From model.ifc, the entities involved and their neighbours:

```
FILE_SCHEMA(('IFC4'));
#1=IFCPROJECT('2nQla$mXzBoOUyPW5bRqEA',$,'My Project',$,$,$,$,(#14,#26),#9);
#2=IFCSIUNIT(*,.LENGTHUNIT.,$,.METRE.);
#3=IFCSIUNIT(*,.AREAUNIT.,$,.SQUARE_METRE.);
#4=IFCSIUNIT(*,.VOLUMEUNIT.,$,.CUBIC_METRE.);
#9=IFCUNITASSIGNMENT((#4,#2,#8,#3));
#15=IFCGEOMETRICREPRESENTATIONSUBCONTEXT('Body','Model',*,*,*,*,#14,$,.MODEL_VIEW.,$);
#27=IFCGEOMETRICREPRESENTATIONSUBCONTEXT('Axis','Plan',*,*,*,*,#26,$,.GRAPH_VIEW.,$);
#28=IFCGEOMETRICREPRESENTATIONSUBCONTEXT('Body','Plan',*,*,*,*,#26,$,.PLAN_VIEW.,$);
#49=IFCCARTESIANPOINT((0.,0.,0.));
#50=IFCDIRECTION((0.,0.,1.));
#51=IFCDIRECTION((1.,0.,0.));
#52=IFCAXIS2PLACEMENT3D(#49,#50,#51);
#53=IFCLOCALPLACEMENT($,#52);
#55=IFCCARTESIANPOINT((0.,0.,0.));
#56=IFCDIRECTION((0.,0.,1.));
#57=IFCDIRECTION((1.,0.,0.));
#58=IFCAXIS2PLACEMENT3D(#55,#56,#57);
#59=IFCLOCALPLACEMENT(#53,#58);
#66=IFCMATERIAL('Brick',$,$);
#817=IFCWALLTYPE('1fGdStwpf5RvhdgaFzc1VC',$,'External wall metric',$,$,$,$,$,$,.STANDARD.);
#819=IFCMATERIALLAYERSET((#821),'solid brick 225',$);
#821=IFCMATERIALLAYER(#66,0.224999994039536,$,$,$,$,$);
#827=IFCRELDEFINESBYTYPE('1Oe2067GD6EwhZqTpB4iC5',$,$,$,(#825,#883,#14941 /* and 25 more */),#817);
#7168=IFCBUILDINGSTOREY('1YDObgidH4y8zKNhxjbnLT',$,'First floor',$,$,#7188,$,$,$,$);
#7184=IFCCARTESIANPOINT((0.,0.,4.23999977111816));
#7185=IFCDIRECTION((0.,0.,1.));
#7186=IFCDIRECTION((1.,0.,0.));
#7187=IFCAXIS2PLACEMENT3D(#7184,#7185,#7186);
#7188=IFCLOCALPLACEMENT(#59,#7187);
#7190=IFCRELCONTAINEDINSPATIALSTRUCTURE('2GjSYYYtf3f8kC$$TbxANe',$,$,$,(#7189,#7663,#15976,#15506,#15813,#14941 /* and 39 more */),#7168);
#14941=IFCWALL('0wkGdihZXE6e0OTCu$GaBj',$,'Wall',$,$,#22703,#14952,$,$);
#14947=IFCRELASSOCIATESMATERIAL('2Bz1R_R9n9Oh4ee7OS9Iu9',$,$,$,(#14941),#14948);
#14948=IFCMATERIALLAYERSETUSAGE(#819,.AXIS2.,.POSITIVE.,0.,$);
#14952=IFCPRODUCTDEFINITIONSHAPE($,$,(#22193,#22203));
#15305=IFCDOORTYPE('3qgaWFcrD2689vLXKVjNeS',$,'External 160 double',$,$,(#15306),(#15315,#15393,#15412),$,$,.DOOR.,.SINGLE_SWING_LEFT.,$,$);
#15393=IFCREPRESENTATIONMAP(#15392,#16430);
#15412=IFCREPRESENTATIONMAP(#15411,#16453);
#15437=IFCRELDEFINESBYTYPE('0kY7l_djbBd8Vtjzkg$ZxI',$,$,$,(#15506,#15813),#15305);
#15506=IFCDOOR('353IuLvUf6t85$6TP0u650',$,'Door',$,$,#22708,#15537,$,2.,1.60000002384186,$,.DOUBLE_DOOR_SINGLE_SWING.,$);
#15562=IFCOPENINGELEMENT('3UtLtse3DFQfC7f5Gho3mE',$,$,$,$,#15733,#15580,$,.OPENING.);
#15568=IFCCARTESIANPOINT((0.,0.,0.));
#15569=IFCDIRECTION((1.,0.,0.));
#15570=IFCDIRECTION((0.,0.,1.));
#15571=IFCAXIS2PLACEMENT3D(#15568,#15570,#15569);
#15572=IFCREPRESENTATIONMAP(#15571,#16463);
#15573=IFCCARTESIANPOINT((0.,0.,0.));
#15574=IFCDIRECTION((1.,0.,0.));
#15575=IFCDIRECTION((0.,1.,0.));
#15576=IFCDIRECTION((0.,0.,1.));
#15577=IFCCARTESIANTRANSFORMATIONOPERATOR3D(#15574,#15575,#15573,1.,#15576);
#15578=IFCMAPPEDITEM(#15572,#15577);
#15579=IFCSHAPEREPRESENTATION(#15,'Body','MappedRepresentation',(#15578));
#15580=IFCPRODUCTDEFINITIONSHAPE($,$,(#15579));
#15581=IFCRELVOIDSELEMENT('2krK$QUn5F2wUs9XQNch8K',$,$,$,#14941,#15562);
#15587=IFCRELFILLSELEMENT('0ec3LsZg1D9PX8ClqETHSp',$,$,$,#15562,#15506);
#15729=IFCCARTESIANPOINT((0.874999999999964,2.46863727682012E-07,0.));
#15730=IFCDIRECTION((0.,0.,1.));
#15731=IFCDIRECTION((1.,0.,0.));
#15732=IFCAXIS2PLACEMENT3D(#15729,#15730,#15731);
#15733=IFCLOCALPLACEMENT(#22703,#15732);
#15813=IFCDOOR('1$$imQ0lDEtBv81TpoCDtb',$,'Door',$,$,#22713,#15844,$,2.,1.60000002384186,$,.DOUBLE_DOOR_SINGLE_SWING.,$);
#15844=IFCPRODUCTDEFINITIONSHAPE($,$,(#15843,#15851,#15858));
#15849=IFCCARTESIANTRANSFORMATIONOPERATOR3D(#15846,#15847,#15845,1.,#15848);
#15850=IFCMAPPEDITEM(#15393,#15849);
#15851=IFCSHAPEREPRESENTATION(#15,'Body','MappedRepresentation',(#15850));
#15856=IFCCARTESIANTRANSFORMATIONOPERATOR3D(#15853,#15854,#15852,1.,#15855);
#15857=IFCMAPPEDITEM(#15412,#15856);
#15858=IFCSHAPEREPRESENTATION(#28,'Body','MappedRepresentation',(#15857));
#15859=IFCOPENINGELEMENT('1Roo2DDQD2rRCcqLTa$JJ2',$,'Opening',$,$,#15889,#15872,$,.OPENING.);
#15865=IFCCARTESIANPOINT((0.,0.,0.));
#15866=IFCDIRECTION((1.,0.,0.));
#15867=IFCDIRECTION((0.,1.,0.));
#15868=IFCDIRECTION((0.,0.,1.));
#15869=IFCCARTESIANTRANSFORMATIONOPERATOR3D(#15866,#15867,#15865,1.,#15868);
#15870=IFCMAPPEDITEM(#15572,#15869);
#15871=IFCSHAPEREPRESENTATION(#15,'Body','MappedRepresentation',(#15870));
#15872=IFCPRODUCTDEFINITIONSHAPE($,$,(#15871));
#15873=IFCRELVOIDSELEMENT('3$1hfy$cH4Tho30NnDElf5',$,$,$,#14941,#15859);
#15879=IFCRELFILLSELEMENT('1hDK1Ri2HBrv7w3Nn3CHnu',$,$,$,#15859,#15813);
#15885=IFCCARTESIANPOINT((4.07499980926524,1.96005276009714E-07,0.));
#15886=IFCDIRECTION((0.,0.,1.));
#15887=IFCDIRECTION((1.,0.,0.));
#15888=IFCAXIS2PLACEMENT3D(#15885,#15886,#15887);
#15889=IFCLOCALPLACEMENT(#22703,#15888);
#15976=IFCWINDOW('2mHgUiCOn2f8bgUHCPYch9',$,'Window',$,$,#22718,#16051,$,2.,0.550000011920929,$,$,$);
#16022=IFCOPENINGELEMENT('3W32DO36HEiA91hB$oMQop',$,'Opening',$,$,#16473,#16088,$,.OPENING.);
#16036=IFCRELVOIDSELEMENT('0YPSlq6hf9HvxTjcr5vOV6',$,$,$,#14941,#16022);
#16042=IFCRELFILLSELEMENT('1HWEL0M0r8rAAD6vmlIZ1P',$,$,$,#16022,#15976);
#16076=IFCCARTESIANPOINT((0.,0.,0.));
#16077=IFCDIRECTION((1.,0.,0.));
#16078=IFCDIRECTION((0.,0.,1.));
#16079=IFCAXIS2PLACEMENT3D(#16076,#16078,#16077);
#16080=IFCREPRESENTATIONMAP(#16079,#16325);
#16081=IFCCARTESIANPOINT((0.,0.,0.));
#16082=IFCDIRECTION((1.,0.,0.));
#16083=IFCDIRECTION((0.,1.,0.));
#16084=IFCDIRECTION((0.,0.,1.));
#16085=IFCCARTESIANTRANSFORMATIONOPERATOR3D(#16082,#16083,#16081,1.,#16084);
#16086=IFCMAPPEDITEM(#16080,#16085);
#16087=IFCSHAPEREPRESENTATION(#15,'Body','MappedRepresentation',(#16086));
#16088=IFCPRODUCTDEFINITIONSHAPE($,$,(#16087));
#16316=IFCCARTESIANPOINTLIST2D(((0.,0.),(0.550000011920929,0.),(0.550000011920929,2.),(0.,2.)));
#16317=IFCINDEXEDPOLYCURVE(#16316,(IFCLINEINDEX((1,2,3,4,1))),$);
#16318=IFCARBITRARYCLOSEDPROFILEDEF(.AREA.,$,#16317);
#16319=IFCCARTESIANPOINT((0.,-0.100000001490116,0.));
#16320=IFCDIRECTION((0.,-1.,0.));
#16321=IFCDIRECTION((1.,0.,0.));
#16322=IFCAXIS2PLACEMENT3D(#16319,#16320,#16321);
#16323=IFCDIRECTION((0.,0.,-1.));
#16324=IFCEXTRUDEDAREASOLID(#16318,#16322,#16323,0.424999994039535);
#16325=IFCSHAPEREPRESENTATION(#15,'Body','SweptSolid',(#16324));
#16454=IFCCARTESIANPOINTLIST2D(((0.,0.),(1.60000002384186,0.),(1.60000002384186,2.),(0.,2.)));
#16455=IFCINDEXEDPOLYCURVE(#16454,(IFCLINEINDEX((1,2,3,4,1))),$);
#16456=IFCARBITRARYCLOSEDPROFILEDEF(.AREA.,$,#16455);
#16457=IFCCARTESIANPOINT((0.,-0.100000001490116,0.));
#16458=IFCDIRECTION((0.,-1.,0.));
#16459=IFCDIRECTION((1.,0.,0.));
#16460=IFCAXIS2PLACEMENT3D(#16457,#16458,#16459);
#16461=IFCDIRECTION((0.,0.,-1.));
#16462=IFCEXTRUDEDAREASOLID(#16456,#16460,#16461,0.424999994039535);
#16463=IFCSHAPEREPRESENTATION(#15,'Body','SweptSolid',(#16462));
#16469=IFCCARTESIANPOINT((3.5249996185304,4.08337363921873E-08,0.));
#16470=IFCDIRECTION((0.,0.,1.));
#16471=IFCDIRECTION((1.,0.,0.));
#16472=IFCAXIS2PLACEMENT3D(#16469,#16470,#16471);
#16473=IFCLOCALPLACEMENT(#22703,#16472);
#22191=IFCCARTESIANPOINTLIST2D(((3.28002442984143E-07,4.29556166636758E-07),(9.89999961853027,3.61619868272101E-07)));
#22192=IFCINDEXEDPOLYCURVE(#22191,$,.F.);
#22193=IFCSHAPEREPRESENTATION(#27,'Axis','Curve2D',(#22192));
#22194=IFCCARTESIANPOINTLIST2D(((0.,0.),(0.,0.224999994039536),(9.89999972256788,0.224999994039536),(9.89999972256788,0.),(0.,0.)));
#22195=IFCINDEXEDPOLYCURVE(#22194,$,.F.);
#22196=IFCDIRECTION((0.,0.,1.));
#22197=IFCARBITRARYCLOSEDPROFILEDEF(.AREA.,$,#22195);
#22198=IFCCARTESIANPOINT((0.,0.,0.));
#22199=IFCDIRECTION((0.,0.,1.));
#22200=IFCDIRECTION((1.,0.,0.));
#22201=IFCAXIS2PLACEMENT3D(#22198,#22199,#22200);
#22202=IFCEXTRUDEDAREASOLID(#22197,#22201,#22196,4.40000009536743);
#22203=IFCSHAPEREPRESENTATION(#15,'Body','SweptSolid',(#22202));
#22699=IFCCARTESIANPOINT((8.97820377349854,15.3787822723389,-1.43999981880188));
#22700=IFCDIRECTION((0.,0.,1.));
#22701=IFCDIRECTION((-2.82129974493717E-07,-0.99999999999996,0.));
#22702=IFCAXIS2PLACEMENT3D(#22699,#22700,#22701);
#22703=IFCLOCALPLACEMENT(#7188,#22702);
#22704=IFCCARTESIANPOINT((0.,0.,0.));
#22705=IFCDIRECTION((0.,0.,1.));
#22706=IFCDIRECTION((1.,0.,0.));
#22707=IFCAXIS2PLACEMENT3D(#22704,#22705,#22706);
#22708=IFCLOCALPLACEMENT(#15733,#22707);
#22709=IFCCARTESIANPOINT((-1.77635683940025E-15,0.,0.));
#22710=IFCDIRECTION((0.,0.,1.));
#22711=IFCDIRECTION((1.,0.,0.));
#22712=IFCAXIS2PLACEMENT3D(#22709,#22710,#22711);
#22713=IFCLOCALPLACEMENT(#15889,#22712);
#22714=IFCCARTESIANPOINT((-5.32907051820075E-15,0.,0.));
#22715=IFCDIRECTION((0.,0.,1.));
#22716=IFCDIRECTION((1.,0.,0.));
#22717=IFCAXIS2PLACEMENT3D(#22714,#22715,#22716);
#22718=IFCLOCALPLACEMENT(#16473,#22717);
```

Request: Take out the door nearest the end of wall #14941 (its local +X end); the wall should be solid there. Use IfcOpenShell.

```python
import ifcopenshell
import ifcopenshell.api.feature
import ifcopenshell.api.root
import ifcopenshell.geom
import ifcopenshell.util.shape

model = ifcopenshell.open("model.ifc")
settings = ifcopenshell.geom.settings()


def volume(element):
    """Net volume in cubic metres, openings subtracted."""
    shape = ifcopenshell.geom.create_shape(settings, element)
    return ifcopenshell.util.shape.get_volume(shape.geometry)


door = model.by_guid("1$$imQ0lDEtBv81TpoCDtb")
opening = door.FillsVoids[0].RelatingOpeningElement
wall = opening.VoidsElements[0].RelatingBuildingElement
before = volume(wall)

ifcopenshell.api.root.remove_product(model, product=door)
ifcopenshell.api.feature.remove_feature(model, feature=opening)

after = volume(wall)

print(f"wall volume {before:.3f} -> {after:.3f} m3")

model.write("model_rev.ifc")
```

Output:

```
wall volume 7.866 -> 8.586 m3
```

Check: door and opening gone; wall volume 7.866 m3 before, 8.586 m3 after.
